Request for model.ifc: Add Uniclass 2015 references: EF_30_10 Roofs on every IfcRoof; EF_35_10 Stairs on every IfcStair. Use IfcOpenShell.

First a look at what the model holds.

```python
import ifcopenshell

model = ifcopenshell.open("model.ifc")
print(model.schema)
print("classifications:", [c.Name for c in model.by_type("IfcClassification")])
for ifc_class in ("IfcDoor", "IfcRoof", "IfcStair", "IfcWall", "IfcWindow"):
    print(ifc_class, len(model.by_type(ifc_class)))
```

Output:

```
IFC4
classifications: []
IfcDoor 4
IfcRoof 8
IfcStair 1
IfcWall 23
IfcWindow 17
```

```python
import ifcopenshell
import ifcopenshell.api.classification

model = ifcopenshell.open("model.ifc")

system = ifcopenshell.api.classification.add_classification(model, classification="Uniclass 2015")

codes = {
    "IfcRoof": ("EF_30_10", "Roofs"),
    "IfcStair": ("EF_35_10", "Stairs"),
}
for ifc_class, (code, name) in codes.items():
    products = model.by_type(ifc_class)
    ifcopenshell.api.classification.add_reference(
        model, products=products, classification=system, identification=code, name=name
    )
    print(code, len(products))

model.write("model_updated.ifc")
```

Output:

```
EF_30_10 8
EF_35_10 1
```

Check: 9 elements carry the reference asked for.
